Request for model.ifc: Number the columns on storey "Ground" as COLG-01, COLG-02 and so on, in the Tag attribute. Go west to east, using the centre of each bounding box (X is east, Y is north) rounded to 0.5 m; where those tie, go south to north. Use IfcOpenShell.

First a look at what the model holds.

```python
import ifcopenshell
import ifcopenshell.util.element
import ifcopenshell.util.placement

model = ifcopenshell.open("model.ifc")
print(model.schema)
storey = next(s for s in model.by_type("IfcBuildingStorey") if s.Name == "Ground")
columns = [e for e in ifcopenshell.util.element.get_decomposition(storey) if e.is_a("IfcColumn")]
for e in sorted(columns, key=lambda e: e.id()):
    origin = ifcopenshell.util.placement.get_local_placement(e.ObjectPlacement)[:3, 3]
    print(e.id(), e.Tag, e.Name, origin.round(2) + 0.0, sep=" | ")
```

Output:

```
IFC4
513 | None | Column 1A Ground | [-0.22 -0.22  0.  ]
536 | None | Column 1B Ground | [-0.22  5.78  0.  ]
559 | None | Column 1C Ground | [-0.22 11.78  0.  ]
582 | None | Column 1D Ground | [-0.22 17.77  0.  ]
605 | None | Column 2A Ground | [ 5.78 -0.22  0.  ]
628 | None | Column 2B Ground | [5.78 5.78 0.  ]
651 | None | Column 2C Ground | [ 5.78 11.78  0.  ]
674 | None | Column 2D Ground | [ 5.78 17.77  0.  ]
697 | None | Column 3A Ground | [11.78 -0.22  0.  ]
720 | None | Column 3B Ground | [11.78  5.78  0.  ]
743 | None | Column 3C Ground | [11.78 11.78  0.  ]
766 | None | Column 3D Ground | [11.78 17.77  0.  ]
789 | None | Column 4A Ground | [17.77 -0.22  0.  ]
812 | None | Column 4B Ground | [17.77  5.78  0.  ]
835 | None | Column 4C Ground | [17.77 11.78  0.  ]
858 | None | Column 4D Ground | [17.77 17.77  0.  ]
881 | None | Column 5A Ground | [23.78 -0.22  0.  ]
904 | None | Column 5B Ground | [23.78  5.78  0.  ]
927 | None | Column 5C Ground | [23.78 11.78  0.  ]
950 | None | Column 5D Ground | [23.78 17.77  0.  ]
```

```python
import ifcopenshell
import ifcopenshell.geom
import ifcopenshell.util.element
import ifcopenshell.util.shape

model = ifcopenshell.open("model.ifc")
settings = ifcopenshell.geom.settings()
settings.set("use-world-coords", True)


def centre(element):
    shape = ifcopenshell.geom.create_shape(settings, element)
    return ifcopenshell.util.shape.get_bbox_centroid(shape.geometry)


storey = next(s for s in model.by_type("IfcBuildingStorey") if s.Name == "Ground")
columns = [e for e in ifcopenshell.util.element.get_decomposition(storey) if e.is_a("IfcColumn")]

# Insertion points can sit at a corner or the storey origin, so sort by the geometry (in metres).
centres = {e: centre(e) for e in columns}
columns.sort(key=lambda e: (round(centres[e][0] / 0.5), centres[e][1]))

for i, e in enumerate(columns, start=1):
    number = f"COLG-{i:02d}"
    e.Tag = number
    print(e.id(), number)

model.write("model_updated.ifc")
```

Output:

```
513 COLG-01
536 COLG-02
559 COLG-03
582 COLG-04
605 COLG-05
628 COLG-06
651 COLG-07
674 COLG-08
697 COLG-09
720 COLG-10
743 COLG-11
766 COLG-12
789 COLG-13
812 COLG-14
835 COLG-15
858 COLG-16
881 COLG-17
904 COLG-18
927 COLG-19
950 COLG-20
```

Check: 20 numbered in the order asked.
